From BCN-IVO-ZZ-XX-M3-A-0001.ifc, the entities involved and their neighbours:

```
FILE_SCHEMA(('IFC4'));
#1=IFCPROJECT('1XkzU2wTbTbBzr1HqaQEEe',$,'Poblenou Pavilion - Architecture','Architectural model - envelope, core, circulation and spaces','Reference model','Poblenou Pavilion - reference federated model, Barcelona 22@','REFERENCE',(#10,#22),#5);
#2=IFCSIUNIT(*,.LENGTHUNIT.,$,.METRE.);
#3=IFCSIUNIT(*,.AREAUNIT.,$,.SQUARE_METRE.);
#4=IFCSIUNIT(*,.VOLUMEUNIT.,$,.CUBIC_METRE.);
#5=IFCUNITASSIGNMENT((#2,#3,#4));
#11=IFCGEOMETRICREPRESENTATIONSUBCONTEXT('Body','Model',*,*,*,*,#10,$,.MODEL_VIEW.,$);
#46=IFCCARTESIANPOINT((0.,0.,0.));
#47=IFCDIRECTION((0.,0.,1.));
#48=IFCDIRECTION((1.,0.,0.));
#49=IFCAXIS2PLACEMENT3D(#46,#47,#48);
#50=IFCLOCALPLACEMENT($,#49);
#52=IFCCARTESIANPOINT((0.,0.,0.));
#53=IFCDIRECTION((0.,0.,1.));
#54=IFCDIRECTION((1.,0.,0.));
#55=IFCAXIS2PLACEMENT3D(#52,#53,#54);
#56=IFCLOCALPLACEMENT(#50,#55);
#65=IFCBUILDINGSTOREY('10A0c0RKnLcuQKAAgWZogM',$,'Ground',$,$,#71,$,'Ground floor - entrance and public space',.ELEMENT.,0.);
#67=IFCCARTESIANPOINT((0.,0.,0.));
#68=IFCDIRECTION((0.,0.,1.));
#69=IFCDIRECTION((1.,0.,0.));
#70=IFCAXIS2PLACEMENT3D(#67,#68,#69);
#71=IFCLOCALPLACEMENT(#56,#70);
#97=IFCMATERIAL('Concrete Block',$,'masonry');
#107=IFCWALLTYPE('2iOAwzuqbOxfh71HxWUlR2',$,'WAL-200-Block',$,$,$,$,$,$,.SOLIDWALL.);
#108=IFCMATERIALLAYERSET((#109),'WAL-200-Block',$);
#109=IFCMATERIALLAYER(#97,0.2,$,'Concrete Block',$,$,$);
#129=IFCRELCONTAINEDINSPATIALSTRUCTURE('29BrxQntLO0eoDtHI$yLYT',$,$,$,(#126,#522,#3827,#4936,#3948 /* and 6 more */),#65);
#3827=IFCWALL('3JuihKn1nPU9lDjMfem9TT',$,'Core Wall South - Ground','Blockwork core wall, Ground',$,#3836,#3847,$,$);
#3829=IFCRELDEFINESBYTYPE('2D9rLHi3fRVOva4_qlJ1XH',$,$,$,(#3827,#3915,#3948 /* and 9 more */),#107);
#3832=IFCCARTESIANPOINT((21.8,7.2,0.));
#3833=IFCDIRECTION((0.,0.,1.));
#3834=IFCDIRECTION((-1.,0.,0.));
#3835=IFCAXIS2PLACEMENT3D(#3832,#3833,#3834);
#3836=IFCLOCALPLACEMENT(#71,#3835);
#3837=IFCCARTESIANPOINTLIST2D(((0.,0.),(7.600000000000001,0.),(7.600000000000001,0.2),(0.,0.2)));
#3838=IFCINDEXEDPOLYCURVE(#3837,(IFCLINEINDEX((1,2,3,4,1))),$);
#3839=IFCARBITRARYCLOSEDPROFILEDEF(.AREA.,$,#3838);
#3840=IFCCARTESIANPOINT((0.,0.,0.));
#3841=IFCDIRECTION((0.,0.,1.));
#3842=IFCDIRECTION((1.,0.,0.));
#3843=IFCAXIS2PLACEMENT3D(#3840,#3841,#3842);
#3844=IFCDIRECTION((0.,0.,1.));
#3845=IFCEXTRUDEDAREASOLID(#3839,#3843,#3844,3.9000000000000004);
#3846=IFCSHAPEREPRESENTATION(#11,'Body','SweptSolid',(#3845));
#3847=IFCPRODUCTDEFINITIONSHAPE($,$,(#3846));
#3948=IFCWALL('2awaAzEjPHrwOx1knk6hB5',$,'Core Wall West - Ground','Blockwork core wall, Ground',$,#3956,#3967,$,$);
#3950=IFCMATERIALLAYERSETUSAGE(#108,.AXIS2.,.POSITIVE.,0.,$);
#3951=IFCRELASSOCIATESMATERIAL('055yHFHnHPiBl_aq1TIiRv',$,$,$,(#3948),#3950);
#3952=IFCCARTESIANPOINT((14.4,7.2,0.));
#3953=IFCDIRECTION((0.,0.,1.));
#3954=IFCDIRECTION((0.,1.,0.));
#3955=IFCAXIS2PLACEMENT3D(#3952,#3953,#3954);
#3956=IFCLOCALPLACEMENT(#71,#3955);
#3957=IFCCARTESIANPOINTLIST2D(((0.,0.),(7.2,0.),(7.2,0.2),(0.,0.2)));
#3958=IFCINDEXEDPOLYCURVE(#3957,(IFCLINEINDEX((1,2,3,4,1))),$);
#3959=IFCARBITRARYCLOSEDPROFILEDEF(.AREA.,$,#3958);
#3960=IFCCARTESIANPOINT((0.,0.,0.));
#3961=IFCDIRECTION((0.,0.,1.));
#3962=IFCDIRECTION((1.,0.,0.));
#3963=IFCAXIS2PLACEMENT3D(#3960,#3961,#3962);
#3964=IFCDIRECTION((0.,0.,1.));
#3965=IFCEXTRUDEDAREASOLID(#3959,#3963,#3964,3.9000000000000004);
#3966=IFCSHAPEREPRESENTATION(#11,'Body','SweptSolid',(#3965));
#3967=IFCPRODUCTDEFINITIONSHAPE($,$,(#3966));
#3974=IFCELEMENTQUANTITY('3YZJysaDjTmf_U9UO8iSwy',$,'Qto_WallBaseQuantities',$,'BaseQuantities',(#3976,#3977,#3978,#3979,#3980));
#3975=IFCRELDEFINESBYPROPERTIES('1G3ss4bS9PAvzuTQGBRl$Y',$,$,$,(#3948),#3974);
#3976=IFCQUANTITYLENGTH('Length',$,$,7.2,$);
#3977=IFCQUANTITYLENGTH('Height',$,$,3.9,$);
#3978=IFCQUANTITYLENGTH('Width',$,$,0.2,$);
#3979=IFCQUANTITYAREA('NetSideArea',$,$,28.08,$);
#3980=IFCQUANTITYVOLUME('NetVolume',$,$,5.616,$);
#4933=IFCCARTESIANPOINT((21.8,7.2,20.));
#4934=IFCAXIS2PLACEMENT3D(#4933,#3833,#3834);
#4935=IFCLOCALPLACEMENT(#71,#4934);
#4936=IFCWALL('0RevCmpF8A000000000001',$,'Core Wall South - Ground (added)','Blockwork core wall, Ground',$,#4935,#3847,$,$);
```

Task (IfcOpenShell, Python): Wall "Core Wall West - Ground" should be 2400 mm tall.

```python
import ifcopenshell
import ifcopenshell.api.pset
import ifcopenshell.geom
import ifcopenshell.util.element
import ifcopenshell.util.representation
import ifcopenshell.util.shape
import ifcopenshell.util.unit

model = ifcopenshell.open("BCN-IVO-ZZ-XX-M3-A-0001.ifc")
unit_scale = ifcopenshell.util.unit.calculate_unit_scale(model)
area_scale = ifcopenshell.util.unit.calculate_unit_scale(model, "AREAUNIT")
volume_scale = ifcopenshell.util.unit.calculate_unit_scale(model, "VOLUMEUNIT")
settings = ifcopenshell.geom.settings()


def volume(element):
    """Net volume in cubic metres, openings subtracted."""
    shape = ifcopenshell.geom.create_shape(settings, element)
    return ifcopenshell.util.shape.get_volume(shape.geometry)


wall = model.by_guid("2awaAzEjPHrwOx1knk6hB5")
before = volume(wall)

body = ifcopenshell.util.representation.get_representation(wall, "Model", "Body")
solid = body.Items[0]
old_height = solid.Depth
solid.Depth = 2.4 / unit_scale
after = volume(wall)
thickness = 0.2  # wall thickness in metres

# Update the stored height, areas and volumes.
qto = model.by_id(ifcopenshell.util.element.get_pset(wall, "Qto_WallBaseQuantities", should_inherit=False)["id"])
ifcopenshell.api.pset.edit_qto(model, qto=qto, properties={
    "Height": solid.Depth,
    "NetSideArea": after / thickness / area_scale,
    "NetVolume": after / volume_scale,
})

print(f"height {old_height:g} -> {solid.Depth:g}, volume {before:.3f} -> {after:.3f} m3")

model.write("BCN-IVO-ZZ-XX-M3-A-0001_v2.ifc")
```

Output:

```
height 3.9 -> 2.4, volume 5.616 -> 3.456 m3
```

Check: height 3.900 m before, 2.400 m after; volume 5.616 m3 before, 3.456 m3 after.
